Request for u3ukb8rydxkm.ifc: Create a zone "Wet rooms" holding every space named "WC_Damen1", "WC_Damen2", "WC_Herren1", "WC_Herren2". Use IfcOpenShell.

First a look at what the model holds.

```python
import ifcopenshell

model = ifcopenshell.open("u3ukb8rydxkm.ifc")
print(model.schema)
seen = {}
for space in model.by_type("IfcSpace"):
    seen[space.Name] = seen.get(space.Name, 0) + 1
for name, count in sorted(seen.items(), key=str):
    print(count, "x", name)
print("zones:", [z.Name for z in model.by_type("IfcZone")][:20])
```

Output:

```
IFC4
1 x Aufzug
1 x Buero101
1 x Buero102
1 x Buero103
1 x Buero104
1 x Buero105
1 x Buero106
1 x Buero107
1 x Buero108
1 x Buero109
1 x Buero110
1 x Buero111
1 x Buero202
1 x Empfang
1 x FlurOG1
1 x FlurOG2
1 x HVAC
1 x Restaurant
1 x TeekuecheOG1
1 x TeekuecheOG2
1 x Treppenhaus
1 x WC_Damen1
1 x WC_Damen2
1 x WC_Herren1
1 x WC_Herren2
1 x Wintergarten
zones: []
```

```python
import ifcopenshell
import ifcopenshell.api.group
import ifcopenshell.api.root

model = ifcopenshell.open("u3ukb8rydxkm.ifc")

names = {"WC_Damen1", "WC_Damen2", "WC_Herren1", "WC_Herren2"}
spaces = [s for s in model.by_type("IfcSpace") if s.Name in names]

zone = ifcopenshell.api.root.create_entity(model, ifc_class="IfcZone", name="Wet rooms")
ifcopenshell.api.group.assign_group(model, products=spaces, group=zone)
print(len(spaces), "spaces in", zone.Name)

model.write("u3ukb8rydxkm_updated.ifc")
```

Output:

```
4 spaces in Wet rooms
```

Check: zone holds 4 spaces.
